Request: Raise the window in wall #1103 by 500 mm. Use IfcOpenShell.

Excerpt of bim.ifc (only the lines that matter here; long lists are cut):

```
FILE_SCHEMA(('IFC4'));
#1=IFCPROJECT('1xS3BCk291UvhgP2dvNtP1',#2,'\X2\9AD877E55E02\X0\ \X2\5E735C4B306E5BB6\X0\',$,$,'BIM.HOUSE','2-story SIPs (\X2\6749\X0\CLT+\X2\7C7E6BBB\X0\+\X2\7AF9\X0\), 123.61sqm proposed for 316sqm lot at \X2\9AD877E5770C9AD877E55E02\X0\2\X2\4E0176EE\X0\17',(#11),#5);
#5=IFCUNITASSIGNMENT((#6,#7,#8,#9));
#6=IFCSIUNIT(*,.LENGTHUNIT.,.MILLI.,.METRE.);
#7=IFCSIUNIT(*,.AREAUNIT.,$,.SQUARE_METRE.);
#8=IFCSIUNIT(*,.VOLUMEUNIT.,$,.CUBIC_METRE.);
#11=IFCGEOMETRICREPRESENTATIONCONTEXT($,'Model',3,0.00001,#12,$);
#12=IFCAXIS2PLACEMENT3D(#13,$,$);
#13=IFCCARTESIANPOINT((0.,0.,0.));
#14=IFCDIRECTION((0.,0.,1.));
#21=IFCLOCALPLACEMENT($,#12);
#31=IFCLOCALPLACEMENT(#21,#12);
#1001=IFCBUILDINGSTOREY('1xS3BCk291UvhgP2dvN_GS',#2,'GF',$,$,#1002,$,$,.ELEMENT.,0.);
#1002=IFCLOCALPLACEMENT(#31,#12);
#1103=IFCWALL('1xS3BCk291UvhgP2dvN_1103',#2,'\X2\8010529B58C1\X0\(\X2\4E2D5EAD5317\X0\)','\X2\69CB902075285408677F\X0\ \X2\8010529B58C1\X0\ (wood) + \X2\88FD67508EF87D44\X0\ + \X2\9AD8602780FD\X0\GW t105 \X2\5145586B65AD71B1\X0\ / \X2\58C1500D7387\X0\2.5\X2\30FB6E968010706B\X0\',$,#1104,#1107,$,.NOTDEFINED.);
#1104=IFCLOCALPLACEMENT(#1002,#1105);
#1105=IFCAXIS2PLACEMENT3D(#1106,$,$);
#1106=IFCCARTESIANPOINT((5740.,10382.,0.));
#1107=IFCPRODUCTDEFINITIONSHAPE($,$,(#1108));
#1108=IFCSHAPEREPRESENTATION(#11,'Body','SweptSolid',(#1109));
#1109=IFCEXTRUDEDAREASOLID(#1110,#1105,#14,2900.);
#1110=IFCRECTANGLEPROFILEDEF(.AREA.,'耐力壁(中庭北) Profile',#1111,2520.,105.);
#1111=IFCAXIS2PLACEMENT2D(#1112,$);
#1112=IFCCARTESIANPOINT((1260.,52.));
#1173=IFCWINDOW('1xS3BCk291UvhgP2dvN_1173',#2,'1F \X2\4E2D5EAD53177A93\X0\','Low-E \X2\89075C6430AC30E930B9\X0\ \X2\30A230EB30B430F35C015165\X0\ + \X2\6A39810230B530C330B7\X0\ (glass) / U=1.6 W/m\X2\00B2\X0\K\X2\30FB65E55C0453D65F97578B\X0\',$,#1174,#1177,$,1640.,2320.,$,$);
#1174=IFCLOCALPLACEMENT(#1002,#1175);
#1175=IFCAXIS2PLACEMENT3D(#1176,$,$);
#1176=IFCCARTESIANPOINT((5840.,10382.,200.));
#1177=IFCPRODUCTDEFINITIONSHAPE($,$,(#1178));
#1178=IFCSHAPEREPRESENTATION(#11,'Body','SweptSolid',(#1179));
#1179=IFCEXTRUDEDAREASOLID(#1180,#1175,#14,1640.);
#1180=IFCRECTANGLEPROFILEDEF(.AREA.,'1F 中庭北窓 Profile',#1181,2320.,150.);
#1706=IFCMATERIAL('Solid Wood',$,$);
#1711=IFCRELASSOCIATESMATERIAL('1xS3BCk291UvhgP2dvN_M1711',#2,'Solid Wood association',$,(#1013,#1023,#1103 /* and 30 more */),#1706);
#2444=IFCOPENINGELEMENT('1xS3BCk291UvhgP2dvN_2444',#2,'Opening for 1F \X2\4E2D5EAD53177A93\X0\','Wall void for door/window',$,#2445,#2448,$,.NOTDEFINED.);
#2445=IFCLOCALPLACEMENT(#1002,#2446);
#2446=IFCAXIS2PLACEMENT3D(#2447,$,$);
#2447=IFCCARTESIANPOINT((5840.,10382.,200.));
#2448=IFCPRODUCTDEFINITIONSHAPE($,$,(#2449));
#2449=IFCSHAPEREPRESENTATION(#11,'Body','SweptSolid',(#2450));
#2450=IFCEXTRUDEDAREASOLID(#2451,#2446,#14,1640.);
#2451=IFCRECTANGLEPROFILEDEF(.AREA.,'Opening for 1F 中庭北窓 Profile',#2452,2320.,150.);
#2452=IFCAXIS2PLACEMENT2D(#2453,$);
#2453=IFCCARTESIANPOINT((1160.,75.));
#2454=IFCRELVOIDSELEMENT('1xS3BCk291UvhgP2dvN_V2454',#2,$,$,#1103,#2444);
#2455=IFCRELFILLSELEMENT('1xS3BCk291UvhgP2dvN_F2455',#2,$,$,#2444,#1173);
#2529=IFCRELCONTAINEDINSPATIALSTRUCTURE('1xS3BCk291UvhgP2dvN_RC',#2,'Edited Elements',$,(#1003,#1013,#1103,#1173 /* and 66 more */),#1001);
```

```python
import numpy as np
import ifcopenshell
import ifcopenshell.api.geometry
import ifcopenshell.util.placement
import ifcopenshell.util.unit

model = ifcopenshell.open("bim.ifc")
unit_scale = ifcopenshell.util.unit.calculate_unit_scale(model)

window = model.by_guid("1xS3BCk291UvhgP2dvN_1173")
opening = window.FillsVoids[0].RelatingOpeningElement
dz = 0.5 / unit_scale

shift = np.array([0.0, 0.0, dz])
# The window is not placed relative to its opening, so move both.
for product in (opening, window):
    matrix = ifcopenshell.util.placement.get_local_placement(product.ObjectPlacement)
    matrix[:3, 3] += shift
    ifcopenshell.api.geometry.edit_object_placement(model, product=product, matrix=matrix, is_si=False)

print(f"moved by {dz * unit_scale:+.3f} m")

model.write("bim_v2.ifc")
```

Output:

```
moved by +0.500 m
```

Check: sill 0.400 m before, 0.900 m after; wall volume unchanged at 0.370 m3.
